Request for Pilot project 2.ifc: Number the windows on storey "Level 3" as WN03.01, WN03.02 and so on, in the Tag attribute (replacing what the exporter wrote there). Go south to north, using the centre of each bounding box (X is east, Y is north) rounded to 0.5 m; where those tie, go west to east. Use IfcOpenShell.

First a look at what the model holds.

```python
import ifcopenshell
import ifcopenshell.util.element
import ifcopenshell.util.placement

model = ifcopenshell.open("Pilot project 2.ifc")
print(model.schema)
storey = next(s for s in model.by_type("IfcBuildingStorey") if s.Name == "Level 3")
windows = [e for e in ifcopenshell.util.element.get_decomposition(storey) if e.is_a("IfcWindow")]
for e in sorted(windows, key=lambda e: e.id()):
    origin = ifcopenshell.util.placement.get_local_placement(e.ObjectPlacement)[:3, 3]
    print(e.id(), e.Tag, e.Name, origin.round(2) + 0.0, sep=" | ")
```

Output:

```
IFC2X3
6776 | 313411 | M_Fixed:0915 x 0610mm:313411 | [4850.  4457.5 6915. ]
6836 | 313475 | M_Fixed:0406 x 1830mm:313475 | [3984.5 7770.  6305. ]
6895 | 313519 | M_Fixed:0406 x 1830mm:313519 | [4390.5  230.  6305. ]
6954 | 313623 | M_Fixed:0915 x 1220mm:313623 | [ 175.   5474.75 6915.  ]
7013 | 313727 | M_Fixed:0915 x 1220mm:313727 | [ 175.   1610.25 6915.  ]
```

```python
import ifcopenshell
import ifcopenshell.geom
import ifcopenshell.util.element
import ifcopenshell.util.shape

model = ifcopenshell.open("Pilot project 2.ifc")
settings = ifcopenshell.geom.settings()
settings.set("use-world-coords", True)


def centre(element):
    shape = ifcopenshell.geom.create_shape(settings, element)
    return ifcopenshell.util.shape.get_bbox_centroid(shape.geometry)


storey = next(s for s in model.by_type("IfcBuildingStorey") if s.Name == "Level 3")
windows = [e for e in ifcopenshell.util.element.get_decomposition(storey) if e.is_a("IfcWindow")]

# Insertion points can sit at a corner or the storey origin, so sort by the geometry (in metres).
centres = {e: centre(e) for e in windows}
windows.sort(key=lambda e: (round(centres[e][1] / 0.5), centres[e][0]))

for i, e in enumerate(windows, start=1):
    number = f"WN03.{i:02d}"
    e.Tag = number
    print(e.id(), number)

model.write("Pilot project 2_v2.ifc")
```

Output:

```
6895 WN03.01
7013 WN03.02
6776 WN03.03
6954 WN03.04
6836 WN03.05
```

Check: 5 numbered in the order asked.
